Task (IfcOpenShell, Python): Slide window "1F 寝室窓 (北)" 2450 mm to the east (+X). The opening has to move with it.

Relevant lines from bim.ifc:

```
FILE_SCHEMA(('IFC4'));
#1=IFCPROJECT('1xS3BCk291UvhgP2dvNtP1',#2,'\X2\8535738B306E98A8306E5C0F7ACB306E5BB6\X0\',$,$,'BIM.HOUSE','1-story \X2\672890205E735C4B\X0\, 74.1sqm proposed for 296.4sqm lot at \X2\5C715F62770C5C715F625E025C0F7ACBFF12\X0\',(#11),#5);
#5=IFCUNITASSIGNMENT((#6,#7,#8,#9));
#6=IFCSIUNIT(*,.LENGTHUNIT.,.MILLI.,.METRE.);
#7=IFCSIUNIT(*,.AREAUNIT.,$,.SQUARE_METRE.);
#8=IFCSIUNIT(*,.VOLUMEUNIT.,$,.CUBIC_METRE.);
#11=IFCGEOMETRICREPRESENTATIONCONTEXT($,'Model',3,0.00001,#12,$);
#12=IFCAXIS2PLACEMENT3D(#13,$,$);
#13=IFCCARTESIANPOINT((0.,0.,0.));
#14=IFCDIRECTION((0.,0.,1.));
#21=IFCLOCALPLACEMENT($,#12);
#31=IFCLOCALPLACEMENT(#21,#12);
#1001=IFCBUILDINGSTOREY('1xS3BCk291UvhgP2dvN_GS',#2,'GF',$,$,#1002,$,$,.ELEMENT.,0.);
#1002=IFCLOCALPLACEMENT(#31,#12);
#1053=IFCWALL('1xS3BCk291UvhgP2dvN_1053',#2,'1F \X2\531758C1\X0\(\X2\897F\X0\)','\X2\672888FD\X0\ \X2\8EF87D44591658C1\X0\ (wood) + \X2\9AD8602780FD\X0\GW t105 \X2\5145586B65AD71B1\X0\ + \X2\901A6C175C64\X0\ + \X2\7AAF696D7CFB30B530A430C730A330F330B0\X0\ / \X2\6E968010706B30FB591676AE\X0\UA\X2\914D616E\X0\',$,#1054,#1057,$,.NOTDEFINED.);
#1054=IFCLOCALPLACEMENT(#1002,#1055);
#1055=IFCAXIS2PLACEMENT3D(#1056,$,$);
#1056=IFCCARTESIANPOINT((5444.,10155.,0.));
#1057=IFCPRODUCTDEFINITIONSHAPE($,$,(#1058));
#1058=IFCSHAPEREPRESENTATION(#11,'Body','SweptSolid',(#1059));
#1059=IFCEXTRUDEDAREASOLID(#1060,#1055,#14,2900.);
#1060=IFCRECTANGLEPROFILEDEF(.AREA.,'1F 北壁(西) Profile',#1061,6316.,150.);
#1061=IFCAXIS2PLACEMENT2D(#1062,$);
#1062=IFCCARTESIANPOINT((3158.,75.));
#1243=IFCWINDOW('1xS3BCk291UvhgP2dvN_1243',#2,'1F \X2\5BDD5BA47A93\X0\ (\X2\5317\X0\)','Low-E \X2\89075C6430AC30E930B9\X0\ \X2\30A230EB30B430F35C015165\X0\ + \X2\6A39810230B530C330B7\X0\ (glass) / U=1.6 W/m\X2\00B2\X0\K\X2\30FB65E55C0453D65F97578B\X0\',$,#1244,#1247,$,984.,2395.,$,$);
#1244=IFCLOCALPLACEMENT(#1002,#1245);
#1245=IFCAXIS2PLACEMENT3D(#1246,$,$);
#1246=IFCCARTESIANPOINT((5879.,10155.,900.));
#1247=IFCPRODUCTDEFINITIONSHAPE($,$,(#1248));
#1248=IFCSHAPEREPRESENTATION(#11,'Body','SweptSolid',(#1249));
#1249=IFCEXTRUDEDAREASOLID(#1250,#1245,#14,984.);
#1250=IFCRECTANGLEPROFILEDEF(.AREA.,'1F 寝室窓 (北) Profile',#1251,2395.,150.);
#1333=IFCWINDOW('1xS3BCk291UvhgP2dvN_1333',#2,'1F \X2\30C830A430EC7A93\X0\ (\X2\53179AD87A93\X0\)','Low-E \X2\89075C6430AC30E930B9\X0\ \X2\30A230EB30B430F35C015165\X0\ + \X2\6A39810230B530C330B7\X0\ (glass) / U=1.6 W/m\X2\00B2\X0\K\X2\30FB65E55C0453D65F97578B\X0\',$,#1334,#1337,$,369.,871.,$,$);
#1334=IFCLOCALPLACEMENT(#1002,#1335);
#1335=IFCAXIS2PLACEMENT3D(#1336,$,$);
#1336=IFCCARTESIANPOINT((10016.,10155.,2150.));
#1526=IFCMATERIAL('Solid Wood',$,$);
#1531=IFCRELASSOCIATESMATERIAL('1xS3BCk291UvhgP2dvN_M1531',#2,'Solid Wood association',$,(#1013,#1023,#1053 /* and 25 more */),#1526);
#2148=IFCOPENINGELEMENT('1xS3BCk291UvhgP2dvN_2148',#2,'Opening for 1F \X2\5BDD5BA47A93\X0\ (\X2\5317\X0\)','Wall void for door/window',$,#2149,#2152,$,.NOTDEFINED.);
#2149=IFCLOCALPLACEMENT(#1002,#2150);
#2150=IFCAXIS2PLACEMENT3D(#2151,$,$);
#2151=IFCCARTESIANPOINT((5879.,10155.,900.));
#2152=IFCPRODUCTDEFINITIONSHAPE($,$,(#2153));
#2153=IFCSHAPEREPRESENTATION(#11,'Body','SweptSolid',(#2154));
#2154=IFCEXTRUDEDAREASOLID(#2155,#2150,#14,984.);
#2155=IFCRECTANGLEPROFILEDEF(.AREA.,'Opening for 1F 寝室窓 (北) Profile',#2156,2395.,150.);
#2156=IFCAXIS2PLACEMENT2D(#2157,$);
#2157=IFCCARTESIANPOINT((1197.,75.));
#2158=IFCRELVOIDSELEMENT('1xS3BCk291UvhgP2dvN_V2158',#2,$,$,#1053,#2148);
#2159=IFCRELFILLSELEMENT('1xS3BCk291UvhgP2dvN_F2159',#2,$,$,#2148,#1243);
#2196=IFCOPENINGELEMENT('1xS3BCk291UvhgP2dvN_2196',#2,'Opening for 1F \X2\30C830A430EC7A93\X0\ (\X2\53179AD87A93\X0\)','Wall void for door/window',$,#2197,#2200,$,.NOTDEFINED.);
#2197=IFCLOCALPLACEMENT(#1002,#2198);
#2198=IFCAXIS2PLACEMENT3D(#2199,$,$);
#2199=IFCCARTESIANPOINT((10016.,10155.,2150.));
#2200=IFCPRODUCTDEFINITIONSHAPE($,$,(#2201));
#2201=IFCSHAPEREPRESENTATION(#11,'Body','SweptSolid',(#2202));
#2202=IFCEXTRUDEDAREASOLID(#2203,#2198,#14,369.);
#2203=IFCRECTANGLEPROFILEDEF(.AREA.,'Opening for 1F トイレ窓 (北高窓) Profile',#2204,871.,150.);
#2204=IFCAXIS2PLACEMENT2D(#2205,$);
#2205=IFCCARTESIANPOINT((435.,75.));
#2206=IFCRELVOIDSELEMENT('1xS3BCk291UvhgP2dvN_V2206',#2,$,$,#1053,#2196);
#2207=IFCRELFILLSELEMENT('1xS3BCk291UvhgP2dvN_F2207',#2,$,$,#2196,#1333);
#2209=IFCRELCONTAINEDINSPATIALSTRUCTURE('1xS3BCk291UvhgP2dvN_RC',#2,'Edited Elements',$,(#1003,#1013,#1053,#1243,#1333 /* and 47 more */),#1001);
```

```python
import ifcopenshell
import ifcopenshell.api.geometry
import ifcopenshell.util.placement
import ifcopenshell.util.unit

model = ifcopenshell.open("bim.ifc")
unit_scale = ifcopenshell.util.unit.calculate_unit_scale(model)

window = model.by_guid("1xS3BCk291UvhgP2dvN_1243")
opening = window.FillsVoids[0].RelatingOpeningElement
wall = opening.VoidsElements[0].RelatingBuildingElement

wall_matrix = ifcopenshell.util.placement.get_local_placement(wall.ObjectPlacement)
shift = wall_matrix[:3, 0] * 2.45 / unit_scale
before = ifcopenshell.util.placement.get_local_placement(window.ObjectPlacement)[:3, 3].copy()

# The window is not placed relative to its opening, so move both.
for product in (opening, window):
    matrix = ifcopenshell.util.placement.get_local_placement(product.ObjectPlacement)
    matrix[:3, 3] += shift
    ifcopenshell.api.geometry.edit_object_placement(model, product=product, matrix=matrix, is_si=False)

after = ifcopenshell.util.placement.get_local_placement(window.ObjectPlacement)[:3, 3]
print("window moved by", (after - before).round(3) + 0.0)

model.write("bim-out.ifc")
```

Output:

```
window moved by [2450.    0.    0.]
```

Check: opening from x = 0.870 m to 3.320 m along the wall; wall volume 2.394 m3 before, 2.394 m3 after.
